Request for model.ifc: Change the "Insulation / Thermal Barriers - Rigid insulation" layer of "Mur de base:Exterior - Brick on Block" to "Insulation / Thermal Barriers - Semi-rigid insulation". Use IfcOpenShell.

First a look at what the model holds.

```python
import ifcopenshell
import ifcopenshell.util.element

model = ifcopenshell.open("model.ifc")
print(model.schema)
for layer_set in model.by_type("IfcMaterialLayerSet"):
    if layer_set.LayerSetName == "Mur de base:Exterior - Brick on Block":
        for layer in layer_set.MaterialLayers:
            print(layer.id(), layer.Material and layer.Material.Name, layer.LayerThickness, sep=" | ")
        print(len(ifcopenshell.util.element.get_elements_by_material(model, layer_set)), "elements and types use it")
print(sorted(m.Name for m in model.by_type("IfcMaterial") if m.Name)[:60])
```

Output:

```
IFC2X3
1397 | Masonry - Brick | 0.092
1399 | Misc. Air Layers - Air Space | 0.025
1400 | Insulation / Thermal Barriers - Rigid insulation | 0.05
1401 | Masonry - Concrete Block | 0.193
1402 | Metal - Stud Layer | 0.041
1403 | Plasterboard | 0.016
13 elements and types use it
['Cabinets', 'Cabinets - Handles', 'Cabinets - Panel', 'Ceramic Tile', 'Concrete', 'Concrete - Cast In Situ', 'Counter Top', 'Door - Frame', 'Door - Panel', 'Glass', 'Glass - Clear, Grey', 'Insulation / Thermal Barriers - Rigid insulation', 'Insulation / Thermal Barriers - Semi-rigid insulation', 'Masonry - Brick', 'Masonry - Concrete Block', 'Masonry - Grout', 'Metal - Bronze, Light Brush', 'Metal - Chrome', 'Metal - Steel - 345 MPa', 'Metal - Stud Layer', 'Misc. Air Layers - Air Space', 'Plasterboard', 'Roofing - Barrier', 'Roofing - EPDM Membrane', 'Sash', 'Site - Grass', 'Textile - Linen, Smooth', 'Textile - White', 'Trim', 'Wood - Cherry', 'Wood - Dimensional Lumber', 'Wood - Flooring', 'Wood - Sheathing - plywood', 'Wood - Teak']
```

```python
import ifcopenshell
import ifcopenshell.api.material

model = ifcopenshell.open("model.ifc")

layer_set = next(s for s in model.by_type("IfcMaterialLayerSet") if s.LayerSetName == "Mur de base:Exterior - Brick on Block")
layer = next(l for l in layer_set.MaterialLayers if l.Material and l.Material.Name == "Insulation / Thermal Barriers - Rigid insulation")
material = next(m for m in model.by_type("IfcMaterial") if m.Name == "Insulation / Thermal Barriers - Semi-rigid insulation")

# Point this one layer at the other material; renaming the old one would change it everywhere.
ifcopenshell.api.material.edit_layer(model, layer=layer, attributes={}, material=material)

print([l.Material.Name if l.Material else None for l in layer_set.MaterialLayers])

model.write("model_v2.ifc")
```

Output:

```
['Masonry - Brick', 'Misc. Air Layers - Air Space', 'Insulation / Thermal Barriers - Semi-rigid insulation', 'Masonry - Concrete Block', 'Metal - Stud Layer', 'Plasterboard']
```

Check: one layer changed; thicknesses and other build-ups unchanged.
